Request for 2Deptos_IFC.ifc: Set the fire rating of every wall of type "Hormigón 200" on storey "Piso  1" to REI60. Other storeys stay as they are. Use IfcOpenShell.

First a look at what the model holds.

```python
import ifcopenshell
import ifcopenshell.util.element

model = ifcopenshell.open("2Deptos_IFC.ifc")
print(model.schema)
storey = next(s for s in model.by_type("IfcBuildingStorey") if s.Name == "Piso  1")
walls = [e for e in ifcopenshell.util.element.get_decomposition(storey) if e.is_a("IfcWall")]
seen = {}
for e in walls:
    element_type = ifcopenshell.util.element.get_type(e)
    key = (element_type.Name if element_type != e and element_type else None, ifcopenshell.util.element.get_pset(e, "Pset_WallCommon", "FireRating"))
    seen[key] = seen.get(key, 0) + 1
for (name, value), count in sorted(seen.items(), key=str):
    print(count, "x", name, "|", value)
```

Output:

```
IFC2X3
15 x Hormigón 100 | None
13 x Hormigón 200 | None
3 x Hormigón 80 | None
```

```python
import ifcopenshell
import ifcopenshell.api.pset
import ifcopenshell.util.element

model = ifcopenshell.open("2Deptos_IFC.ifc")

storey = next(s for s in model.by_type("IfcBuildingStorey") if s.Name == "Piso  1")
walls = [e for e in ifcopenshell.util.element.get_decomposition(storey) if e.is_a("IfcWall")]

count = 0
for e in walls:
    element_type = ifcopenshell.util.element.get_type(e)
    if element_type in (None, e) or element_type.Name != "Hormigón 200":
        continue
    # add_pset returns the element's existing set when there is one.
    pset = ifcopenshell.api.pset.add_pset(model, product=e, name="Pset_WallCommon")
    ifcopenshell.api.pset.edit_pset(model, pset=pset, properties={"FireRating": "REI60"})
    count += 1

print(count, "walls updated")

model.write("2Deptos_IFC_edited.ifc")
```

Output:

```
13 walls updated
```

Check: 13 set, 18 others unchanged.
